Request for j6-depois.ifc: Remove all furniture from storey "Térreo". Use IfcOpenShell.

First a look at what the model holds.

```python
import ifcopenshell
import ifcopenshell.util.element

model = ifcopenshell.open("j6-depois.ifc")
print(model.schema)
storey = next(s for s in model.by_type("IfcBuildingStorey") if s.Name == "Térreo")
furniture = [e for e in ifcopenshell.util.element.get_decomposition(storey) if e.is_a("IfcFurnishingElement")]
seen = {}
for e in furniture:
    element_type = ifcopenshell.util.element.get_type(e)
    name = element_type.Name if element_type not in (None, e) else None
    seen[name] = seen.get(name, 0) + 1
for name, count in sorted(seen.items(), key=str):
    print(count, "x", name)
```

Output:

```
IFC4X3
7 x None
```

```python
import ifcopenshell
import ifcopenshell.api.root
import ifcopenshell.util.element

model = ifcopenshell.open("j6-depois.ifc")

storey = next(s for s in model.by_type("IfcBuildingStorey") if s.Name == "Térreo")
furniture = [e for e in ifcopenshell.util.element.get_decomposition(storey) if e.is_a("IfcFurnishingElement")]

for e in furniture:
    ifcopenshell.api.root.remove_product(model, product=e)
print(len(furniture), "removed")

model.write("j6-depois_edited.ifc")
```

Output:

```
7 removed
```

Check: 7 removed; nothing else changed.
